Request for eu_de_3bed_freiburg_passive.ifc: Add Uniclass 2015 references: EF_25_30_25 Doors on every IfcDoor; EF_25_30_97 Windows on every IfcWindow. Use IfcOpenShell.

First a look at what the model holds.

```python
import ifcopenshell

model = ifcopenshell.open("eu_de_3bed_freiburg_passive.ifc")
print(model.schema)
print("classifications:", [c.Name for c in model.by_type("IfcClassification")])
for ifc_class in ("IfcDoor", "IfcRoof", "IfcStair", "IfcWall", "IfcWindow"):
    print(ifc_class, len(model.by_type(ifc_class)))
```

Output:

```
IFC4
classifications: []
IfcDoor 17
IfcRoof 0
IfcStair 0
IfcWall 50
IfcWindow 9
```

```python
import ifcopenshell
import ifcopenshell.api.classification

model = ifcopenshell.open("eu_de_3bed_freiburg_passive.ifc")

system = ifcopenshell.api.classification.add_classification(model, classification="Uniclass 2015")

codes = {
    "IfcDoor": ("EF_25_30_25", "Doors"),
    "IfcWindow": ("EF_25_30_97", "Windows"),
}
for ifc_class, (code, name) in codes.items():
    products = model.by_type(ifc_class)
    ifcopenshell.api.classification.add_reference(
        model, products=products, classification=system, identification=code, name=name
    )
    print(code, len(products))

model.write("eu_de_3bed_freiburg_passive_rev.ifc")
```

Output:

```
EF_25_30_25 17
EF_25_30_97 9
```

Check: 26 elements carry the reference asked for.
